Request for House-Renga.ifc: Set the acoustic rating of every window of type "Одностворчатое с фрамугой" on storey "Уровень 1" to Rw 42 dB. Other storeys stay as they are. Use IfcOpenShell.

First a look at what the model holds.

```python
import ifcopenshell
import ifcopenshell.util.element

model = ifcopenshell.open("House-Renga.ifc")
print(model.schema)
storey = next(s for s in model.by_type("IfcBuildingStorey") if s.Name == "Уровень 1")
windows = [e for e in ifcopenshell.util.element.get_decomposition(storey) if e.is_a("IfcWindow")]
seen = {}
for e in windows:
    element_type = ifcopenshell.util.element.get_type(e)
    key = (element_type.Name if element_type != e and element_type else None, ifcopenshell.util.element.get_pset(e, "Pset_WindowCommon", "AcousticRating"))
    seen[key] = seen.get(key, 0) + 1
for (name, value), count in sorted(seen.items(), key=str):
    print(count, "x", name, "|", value)
```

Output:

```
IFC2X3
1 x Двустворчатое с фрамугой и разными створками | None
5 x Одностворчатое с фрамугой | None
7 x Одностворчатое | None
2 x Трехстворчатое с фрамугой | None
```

```python
import ifcopenshell
import ifcopenshell.api.pset
import ifcopenshell.util.element

model = ifcopenshell.open("House-Renga.ifc")

storey = next(s for s in model.by_type("IfcBuildingStorey") if s.Name == "Уровень 1")
windows = [e for e in ifcopenshell.util.element.get_decomposition(storey) if e.is_a("IfcWindow")]

count = 0
for e in windows:
    element_type = ifcopenshell.util.element.get_type(e)
    if element_type in (None, e) or element_type.Name != "Одностворчатое с фрамугой":
        continue
    # add_pset returns the element's existing set when there is one.
    pset = ifcopenshell.api.pset.add_pset(model, product=e, name="Pset_WindowCommon")
    ifcopenshell.api.pset.edit_pset(model, pset=pset, properties={"AcousticRating": "Rw 42 dB"})
    count += 1

print(count, "windows updated")

model.write("House-Renga_v2.ifc")
```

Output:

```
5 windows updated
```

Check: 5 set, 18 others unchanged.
